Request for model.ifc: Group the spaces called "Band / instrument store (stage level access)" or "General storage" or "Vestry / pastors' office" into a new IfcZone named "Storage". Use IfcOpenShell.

First a look at what the model holds.

```python
import ifcopenshell

model = ifcopenshell.open("model.ifc")
print(model.schema)
seen = {}
for space in model.by_type("IfcSpace"):
    seen[space.LongName] = seen.get(space.LongName, 0) + 1
for name, count in sorted(seen.items(), key=str):
    print(count, "x", name)
print("zones:", [z.Name for z in model.by_type("IfcZone")][:20])
```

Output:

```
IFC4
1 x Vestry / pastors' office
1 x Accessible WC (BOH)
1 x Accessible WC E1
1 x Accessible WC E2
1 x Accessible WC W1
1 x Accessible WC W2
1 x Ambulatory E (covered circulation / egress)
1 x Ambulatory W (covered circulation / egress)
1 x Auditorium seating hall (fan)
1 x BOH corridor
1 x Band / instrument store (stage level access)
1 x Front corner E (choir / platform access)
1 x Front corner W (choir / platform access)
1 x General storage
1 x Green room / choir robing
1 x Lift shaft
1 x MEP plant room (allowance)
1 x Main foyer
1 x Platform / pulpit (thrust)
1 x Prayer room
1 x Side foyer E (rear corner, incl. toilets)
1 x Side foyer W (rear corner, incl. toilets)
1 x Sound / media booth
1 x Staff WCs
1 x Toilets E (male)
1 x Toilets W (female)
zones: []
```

```python
import ifcopenshell
import ifcopenshell.api.group
import ifcopenshell.api.root

model = ifcopenshell.open("model.ifc")

names = {"Band / instrument store (stage level access)", "General storage", "Vestry / pastors' office"}
spaces = [s for s in model.by_type("IfcSpace") if s.LongName in names]

zone = ifcopenshell.api.root.create_entity(model, ifc_class="IfcZone", name="Storage")
ifcopenshell.api.group.assign_group(model, products=spaces, group=zone)
print(len(spaces), "spaces in", zone.Name)

model.write("model_rev.ifc")
```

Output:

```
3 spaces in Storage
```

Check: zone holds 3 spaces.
